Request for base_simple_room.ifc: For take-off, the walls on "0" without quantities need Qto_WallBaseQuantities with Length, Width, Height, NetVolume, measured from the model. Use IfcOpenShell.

First a look at what the model holds.

```python
import ifcopenshell
import ifcopenshell.util.element
import ifcopenshell.util.unit

model = ifcopenshell.open("base_simple_room.ifc")
print(model.schema)
for unit_type in ("LENGTHUNIT", "AREAUNIT", "VOLUMEUNIT"):
    print(unit_type, ifcopenshell.util.unit.calculate_unit_scale(model, unit_type))
storey = next(s for s in model.by_type("IfcBuildingStorey") if s.Name == "0")
walls = [e for e in ifcopenshell.util.element.get_decomposition(storey) if e.is_a("IfcWall")]
for e in sorted(walls, key=lambda e: e.id()):
    print(e.id(), e.is_a(), e.Name, list(ifcopenshell.util.element.get_psets(e, qtos_only=True)), sep=" | ")
```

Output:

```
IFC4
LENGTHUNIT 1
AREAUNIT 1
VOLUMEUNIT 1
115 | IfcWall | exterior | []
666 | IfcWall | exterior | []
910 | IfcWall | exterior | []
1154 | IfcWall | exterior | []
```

```python
import ifcopenshell
import ifcopenshell.api.pset
import ifcopenshell.geom
import ifcopenshell.util.element
import ifcopenshell.util.shape
import ifcopenshell.util.unit

model = ifcopenshell.open("base_simple_room.ifc")
unit_scale = ifcopenshell.util.unit.calculate_unit_scale(model)
volume_scale = ifcopenshell.util.unit.calculate_unit_scale(model, "VOLUMEUNIT")
settings = ifcopenshell.geom.settings()

storey = next(s for s in model.by_type("IfcBuildingStorey") if s.Name == "0")
walls = [e for e in ifcopenshell.util.element.get_decomposition(storey) if e.is_a("IfcWall")]

for e in sorted(walls, key=lambda e: e.id()):
    if ifcopenshell.util.element.get_psets(e, qtos_only=True, should_inherit=False):
        continue
    # Geometry comes back in metres, in the element's own axes.
    shape = ifcopenshell.geom.create_shape(settings, e)
    values = {
        "Length": ifcopenshell.util.shape.get_x(shape.geometry) / unit_scale,
        "Width": ifcopenshell.util.shape.get_y(shape.geometry) / unit_scale,
        "Height": ifcopenshell.util.shape.get_z(shape.geometry) / unit_scale,
        "NetVolume": ifcopenshell.util.shape.get_volume(shape.geometry) / volume_scale,
    }
    qto = ifcopenshell.api.pset.add_qto(model, product=e, name="Qto_WallBaseQuantities")
    ifcopenshell.api.pset.edit_qto(model, qto=qto, properties=values)
    print(e.id(), {k: round(v, 3) for k, v in values.items()})

model.write("base_simple_room_v2.ifc")
```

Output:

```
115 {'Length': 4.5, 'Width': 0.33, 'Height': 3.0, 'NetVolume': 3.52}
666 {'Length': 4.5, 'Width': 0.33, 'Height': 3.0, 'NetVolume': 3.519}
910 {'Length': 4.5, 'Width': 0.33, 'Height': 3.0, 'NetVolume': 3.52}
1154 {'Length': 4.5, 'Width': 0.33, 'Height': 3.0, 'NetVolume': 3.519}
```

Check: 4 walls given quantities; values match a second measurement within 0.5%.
